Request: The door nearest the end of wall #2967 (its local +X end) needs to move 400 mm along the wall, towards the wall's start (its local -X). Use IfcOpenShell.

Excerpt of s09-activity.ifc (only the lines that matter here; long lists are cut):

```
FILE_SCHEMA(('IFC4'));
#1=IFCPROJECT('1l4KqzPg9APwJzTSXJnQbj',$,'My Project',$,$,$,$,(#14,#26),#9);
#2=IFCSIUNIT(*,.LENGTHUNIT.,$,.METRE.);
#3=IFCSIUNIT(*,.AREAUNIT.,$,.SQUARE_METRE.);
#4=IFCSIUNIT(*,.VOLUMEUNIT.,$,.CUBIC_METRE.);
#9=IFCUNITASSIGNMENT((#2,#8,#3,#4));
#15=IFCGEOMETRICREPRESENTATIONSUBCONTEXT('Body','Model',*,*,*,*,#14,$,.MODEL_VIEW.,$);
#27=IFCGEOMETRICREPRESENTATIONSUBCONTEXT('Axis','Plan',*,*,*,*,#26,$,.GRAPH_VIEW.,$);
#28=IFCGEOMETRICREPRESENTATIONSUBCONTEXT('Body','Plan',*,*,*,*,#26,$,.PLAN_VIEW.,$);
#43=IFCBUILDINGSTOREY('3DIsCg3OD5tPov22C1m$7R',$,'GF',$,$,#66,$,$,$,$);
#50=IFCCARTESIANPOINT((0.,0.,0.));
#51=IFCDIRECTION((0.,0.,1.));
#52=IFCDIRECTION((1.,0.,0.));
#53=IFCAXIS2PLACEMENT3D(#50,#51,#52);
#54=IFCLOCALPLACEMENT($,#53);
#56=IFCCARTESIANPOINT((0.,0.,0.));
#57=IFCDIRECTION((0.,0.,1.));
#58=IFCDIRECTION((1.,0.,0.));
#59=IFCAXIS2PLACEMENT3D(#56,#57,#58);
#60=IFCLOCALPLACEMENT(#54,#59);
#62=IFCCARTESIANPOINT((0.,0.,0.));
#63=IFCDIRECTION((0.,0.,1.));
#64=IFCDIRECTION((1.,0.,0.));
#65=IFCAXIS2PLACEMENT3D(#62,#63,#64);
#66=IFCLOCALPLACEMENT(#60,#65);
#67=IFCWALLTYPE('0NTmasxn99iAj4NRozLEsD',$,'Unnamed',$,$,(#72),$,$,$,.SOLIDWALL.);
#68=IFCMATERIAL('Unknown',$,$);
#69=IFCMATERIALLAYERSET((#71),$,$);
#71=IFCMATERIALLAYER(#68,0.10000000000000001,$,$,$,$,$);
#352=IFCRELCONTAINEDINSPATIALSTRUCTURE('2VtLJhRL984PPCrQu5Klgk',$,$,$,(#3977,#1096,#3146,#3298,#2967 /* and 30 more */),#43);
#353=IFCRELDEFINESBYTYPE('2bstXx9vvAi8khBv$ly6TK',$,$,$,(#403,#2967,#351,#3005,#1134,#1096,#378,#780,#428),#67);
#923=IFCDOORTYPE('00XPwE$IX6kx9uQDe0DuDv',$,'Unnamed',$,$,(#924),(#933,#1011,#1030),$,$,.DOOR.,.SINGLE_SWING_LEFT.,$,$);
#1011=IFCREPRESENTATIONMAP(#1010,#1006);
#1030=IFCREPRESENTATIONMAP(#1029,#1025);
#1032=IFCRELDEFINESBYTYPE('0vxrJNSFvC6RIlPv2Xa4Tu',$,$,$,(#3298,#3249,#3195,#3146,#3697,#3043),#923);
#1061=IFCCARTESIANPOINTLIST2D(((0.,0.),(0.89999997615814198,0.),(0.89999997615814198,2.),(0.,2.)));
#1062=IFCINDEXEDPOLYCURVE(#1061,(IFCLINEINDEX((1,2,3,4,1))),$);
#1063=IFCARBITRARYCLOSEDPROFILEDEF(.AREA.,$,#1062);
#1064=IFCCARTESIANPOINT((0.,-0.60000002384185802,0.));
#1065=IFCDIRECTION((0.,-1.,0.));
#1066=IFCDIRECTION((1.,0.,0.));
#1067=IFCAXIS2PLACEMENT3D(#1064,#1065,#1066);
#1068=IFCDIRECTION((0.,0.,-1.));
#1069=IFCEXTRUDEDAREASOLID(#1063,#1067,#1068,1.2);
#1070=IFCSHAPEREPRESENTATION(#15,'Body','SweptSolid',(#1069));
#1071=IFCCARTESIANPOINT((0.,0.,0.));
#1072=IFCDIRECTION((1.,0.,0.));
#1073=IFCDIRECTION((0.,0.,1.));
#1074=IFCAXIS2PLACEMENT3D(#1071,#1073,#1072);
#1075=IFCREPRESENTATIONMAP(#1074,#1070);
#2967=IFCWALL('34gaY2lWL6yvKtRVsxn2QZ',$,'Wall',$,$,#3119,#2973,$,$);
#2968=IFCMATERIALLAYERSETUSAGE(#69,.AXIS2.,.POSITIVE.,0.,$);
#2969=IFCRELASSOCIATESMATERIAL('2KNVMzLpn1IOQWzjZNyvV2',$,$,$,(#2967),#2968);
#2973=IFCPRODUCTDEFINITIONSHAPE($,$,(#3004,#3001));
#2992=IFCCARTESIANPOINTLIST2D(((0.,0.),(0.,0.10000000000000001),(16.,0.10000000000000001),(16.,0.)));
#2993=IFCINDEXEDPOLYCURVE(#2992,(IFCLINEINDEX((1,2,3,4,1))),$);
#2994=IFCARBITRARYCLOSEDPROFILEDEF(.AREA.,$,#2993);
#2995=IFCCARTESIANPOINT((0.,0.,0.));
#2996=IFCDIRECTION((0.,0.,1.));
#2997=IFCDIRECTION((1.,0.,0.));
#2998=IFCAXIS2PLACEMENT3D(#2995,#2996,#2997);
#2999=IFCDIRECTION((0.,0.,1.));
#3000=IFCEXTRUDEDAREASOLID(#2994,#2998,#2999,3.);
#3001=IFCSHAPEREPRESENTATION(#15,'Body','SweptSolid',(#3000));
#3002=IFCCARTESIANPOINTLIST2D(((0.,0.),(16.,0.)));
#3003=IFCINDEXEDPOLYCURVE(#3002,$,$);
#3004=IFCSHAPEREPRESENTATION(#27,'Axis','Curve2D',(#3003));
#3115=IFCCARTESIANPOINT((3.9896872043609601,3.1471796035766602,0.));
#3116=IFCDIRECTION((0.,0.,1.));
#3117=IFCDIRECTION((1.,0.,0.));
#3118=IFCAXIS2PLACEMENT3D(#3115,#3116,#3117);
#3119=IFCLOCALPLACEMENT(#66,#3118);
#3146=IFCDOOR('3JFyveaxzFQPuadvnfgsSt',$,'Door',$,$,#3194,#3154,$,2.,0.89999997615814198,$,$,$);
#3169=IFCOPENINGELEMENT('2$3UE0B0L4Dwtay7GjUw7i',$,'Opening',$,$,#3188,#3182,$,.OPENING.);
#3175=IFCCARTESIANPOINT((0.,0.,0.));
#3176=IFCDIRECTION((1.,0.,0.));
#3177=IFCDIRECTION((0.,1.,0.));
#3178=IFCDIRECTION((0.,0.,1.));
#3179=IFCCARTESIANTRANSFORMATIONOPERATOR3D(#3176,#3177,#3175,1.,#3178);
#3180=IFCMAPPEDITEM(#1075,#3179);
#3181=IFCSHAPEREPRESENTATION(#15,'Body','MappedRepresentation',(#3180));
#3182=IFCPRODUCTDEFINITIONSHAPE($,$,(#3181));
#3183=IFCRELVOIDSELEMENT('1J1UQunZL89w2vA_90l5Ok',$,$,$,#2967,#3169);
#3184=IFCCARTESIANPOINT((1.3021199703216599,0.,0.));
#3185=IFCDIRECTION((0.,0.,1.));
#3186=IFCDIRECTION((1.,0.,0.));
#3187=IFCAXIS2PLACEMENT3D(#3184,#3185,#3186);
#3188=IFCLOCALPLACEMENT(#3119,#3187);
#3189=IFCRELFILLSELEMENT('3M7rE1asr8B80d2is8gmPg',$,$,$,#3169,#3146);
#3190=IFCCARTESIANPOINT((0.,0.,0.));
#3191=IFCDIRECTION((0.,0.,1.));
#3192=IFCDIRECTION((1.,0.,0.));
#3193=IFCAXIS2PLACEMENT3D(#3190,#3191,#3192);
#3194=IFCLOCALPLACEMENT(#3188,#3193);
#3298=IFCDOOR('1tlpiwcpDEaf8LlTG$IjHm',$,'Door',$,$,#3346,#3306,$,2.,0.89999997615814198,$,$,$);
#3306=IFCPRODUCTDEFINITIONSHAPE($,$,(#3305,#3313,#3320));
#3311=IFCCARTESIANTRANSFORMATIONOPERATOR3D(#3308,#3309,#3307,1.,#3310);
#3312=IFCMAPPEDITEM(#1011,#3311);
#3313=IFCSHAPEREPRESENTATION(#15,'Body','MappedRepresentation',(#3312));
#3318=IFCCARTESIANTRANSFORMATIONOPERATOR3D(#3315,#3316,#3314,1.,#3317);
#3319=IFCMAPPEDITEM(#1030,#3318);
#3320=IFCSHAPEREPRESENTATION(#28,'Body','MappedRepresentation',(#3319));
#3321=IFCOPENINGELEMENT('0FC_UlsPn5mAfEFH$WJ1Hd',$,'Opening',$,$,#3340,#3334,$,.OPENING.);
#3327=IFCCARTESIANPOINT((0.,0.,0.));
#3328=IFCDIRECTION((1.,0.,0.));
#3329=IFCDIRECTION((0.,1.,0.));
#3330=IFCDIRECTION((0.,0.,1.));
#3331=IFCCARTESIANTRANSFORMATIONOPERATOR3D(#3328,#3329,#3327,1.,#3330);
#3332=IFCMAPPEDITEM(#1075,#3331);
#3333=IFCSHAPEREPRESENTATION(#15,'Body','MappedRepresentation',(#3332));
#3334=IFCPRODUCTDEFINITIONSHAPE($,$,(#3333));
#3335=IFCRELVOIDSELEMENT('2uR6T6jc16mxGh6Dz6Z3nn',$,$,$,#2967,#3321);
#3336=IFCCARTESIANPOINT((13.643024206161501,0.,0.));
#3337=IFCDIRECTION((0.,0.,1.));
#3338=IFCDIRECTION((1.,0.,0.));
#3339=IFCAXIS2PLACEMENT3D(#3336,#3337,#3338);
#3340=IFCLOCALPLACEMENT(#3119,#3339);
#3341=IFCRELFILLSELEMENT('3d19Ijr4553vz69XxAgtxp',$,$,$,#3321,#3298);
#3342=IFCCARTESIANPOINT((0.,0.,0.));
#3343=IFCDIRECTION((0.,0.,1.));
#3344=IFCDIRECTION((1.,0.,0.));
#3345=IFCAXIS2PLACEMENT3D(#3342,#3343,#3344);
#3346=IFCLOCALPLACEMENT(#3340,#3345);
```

```python
import ifcopenshell
import ifcopenshell.api.geometry
import ifcopenshell.util.placement
import ifcopenshell.util.unit

model = ifcopenshell.open("s09-activity.ifc")
unit_scale = ifcopenshell.util.unit.calculate_unit_scale(model)

door = model.by_guid("1tlpiwcpDEaf8LlTG$IjHm")
opening = door.FillsVoids[0].RelatingOpeningElement
wall = opening.VoidsElements[0].RelatingBuildingElement

wall_matrix = ifcopenshell.util.placement.get_local_placement(wall.ObjectPlacement)
shift = wall_matrix[:3, 0] * -0.4 / unit_scale
before = ifcopenshell.util.placement.get_local_placement(door.ObjectPlacement)[:3, 3].copy()

# The door is placed relative to its opening, so it follows when the opening moves.
matrix = ifcopenshell.util.placement.get_local_placement(opening.ObjectPlacement)
matrix[:3, 3] += shift
ifcopenshell.api.geometry.edit_object_placement(
    model, product=opening, matrix=matrix, is_si=False, should_transform_children=True
)

after = ifcopenshell.util.placement.get_local_placement(door.ObjectPlacement)[:3, 3]
print("door moved by", (after - before).round(3) + 0.0)

model.write("s09-activity_updated.ifc")
```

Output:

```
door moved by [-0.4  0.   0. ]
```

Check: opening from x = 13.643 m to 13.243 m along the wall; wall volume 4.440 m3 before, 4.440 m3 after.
